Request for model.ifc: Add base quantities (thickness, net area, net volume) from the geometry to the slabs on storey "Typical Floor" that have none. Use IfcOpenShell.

First a look at what the model holds.

```python
import ifcopenshell
import ifcopenshell.util.element
import ifcopenshell.util.unit

model = ifcopenshell.open("model.ifc")
print(model.schema)
for unit_type in ("LENGTHUNIT", "AREAUNIT", "VOLUMEUNIT"):
    print(unit_type, ifcopenshell.util.unit.calculate_unit_scale(model, unit_type))
storey = next(s for s in model.by_type("IfcBuildingStorey") if s.Name == "Typical Floor")
slabs = [e for e in ifcopenshell.util.element.get_decomposition(storey) if e.is_a("IfcSlab")]
for e in sorted(slabs, key=lambda e: e.id()):
    print(e.id(), e.is_a(), e.Name, list(ifcopenshell.util.element.get_psets(e, qtos_only=True)), sep=" | ")
```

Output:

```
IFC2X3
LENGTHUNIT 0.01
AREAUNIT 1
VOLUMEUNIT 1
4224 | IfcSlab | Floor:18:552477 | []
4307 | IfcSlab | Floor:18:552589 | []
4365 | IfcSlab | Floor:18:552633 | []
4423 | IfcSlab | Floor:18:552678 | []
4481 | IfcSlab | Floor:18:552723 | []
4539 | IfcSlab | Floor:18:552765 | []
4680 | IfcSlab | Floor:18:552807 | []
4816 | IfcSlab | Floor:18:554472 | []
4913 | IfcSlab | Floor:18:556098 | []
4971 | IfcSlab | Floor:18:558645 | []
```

```python
import ifcopenshell
import ifcopenshell.api.pset
import ifcopenshell.geom
import ifcopenshell.util.element
import ifcopenshell.util.shape
import ifcopenshell.util.unit

model = ifcopenshell.open("model.ifc")
unit_scale = ifcopenshell.util.unit.calculate_unit_scale(model)
area_scale = ifcopenshell.util.unit.calculate_unit_scale(model, "AREAUNIT")
volume_scale = ifcopenshell.util.unit.calculate_unit_scale(model, "VOLUMEUNIT")
settings = ifcopenshell.geom.settings()

storey = next(s for s in model.by_type("IfcBuildingStorey") if s.Name == "Typical Floor")
slabs = [e for e in ifcopenshell.util.element.get_decomposition(storey) if e.is_a("IfcSlab")]

for e in sorted(slabs, key=lambda e: e.id()):
    if ifcopenshell.util.element.get_psets(e, qtos_only=True, should_inherit=False):
        continue
    # Geometry comes back in metres, in the element's own axes.
    shape = ifcopenshell.geom.create_shape(settings, e)
    values = {
        "Width": ifcopenshell.util.shape.get_z(shape.geometry) / unit_scale,
        "NetArea": ifcopenshell.util.shape.get_footprint_area(shape.geometry) / area_scale,
        "NetVolume": ifcopenshell.util.shape.get_volume(shape.geometry) / volume_scale,
    }
    qto = ifcopenshell.api.pset.add_qto(model, product=e, name="BaseQuantities")
    ifcopenshell.api.pset.edit_qto(model, qto=qto, properties=values)
    print(e.id(), {k: round(v, 3) for k, v in values.items()})

model.write("model-out.ifc")
```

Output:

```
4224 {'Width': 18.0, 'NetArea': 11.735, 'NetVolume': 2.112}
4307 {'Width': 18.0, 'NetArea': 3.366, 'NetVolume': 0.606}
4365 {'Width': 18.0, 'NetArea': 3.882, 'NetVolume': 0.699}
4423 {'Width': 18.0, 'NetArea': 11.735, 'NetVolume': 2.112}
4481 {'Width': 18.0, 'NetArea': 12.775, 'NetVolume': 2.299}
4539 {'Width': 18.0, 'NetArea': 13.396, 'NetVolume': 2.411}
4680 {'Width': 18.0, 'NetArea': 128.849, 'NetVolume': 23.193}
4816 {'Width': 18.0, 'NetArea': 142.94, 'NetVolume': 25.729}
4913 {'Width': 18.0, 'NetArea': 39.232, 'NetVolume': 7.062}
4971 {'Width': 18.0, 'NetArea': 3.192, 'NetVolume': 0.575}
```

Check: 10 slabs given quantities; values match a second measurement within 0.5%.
